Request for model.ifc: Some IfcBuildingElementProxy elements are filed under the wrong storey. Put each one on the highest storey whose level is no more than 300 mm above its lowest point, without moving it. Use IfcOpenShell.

First a look at what the model holds.

```python
import ifcopenshell
import ifcopenshell.util.element
import ifcopenshell.util.placement

model = ifcopenshell.open("model.ifc")
print(model.schema)
for storey in model.by_type("IfcBuildingStorey"):
    level = ifcopenshell.util.placement.get_storey_elevation(storey)
    count = sum(e.is_a("IfcBuildingElementProxy") for e in ifcopenshell.util.element.get_contained(storey))
    print(storey.id(), storey.Name, round(level, 3), count, sep=" | ")
```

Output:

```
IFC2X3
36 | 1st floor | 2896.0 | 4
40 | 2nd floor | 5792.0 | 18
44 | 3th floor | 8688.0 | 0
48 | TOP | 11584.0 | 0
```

```python
import ifcopenshell
import ifcopenshell.api.spatial
import ifcopenshell.geom
import ifcopenshell.util.element
import ifcopenshell.util.placement
import ifcopenshell.util.shape
import ifcopenshell.util.unit

model = ifcopenshell.open("model.ifc")
unit_scale = ifcopenshell.util.unit.calculate_unit_scale(model)
settings = ifcopenshell.geom.settings()

levels = sorted(
    ((ifcopenshell.util.placement.get_storey_elevation(s) * unit_scale, s) for s in model.by_type("IfcBuildingStorey")),
    key=lambda pair: pair[0],
)

for e in model.by_type("IfcBuildingElementProxy"):
    current = e.ContainedInStructure[0].RelatingStructure if e.ContainedInStructure else None
    if current is None or not current.is_a("IfcBuildingStorey"):
        continue
    shape = ifcopenshell.geom.create_shape(settings, e)
    bottom = ifcopenshell.util.shape.get_shape_bottom_elevation(shape, shape.geometry)
    below = [s for level, s in levels if level <= bottom + 0.3]
    storey = below[-1] if below else levels[0][1]
    if storey != current:
        # assign_container keeps the world position.
        ifcopenshell.api.spatial.assign_container(model, products=[e], relating_structure=storey)
        print(e.id(), current.Name, "->", storey.Name)

model.write("model_rev.ifc")
```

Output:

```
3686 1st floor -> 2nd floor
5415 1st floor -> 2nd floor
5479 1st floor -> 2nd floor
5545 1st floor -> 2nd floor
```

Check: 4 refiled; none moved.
